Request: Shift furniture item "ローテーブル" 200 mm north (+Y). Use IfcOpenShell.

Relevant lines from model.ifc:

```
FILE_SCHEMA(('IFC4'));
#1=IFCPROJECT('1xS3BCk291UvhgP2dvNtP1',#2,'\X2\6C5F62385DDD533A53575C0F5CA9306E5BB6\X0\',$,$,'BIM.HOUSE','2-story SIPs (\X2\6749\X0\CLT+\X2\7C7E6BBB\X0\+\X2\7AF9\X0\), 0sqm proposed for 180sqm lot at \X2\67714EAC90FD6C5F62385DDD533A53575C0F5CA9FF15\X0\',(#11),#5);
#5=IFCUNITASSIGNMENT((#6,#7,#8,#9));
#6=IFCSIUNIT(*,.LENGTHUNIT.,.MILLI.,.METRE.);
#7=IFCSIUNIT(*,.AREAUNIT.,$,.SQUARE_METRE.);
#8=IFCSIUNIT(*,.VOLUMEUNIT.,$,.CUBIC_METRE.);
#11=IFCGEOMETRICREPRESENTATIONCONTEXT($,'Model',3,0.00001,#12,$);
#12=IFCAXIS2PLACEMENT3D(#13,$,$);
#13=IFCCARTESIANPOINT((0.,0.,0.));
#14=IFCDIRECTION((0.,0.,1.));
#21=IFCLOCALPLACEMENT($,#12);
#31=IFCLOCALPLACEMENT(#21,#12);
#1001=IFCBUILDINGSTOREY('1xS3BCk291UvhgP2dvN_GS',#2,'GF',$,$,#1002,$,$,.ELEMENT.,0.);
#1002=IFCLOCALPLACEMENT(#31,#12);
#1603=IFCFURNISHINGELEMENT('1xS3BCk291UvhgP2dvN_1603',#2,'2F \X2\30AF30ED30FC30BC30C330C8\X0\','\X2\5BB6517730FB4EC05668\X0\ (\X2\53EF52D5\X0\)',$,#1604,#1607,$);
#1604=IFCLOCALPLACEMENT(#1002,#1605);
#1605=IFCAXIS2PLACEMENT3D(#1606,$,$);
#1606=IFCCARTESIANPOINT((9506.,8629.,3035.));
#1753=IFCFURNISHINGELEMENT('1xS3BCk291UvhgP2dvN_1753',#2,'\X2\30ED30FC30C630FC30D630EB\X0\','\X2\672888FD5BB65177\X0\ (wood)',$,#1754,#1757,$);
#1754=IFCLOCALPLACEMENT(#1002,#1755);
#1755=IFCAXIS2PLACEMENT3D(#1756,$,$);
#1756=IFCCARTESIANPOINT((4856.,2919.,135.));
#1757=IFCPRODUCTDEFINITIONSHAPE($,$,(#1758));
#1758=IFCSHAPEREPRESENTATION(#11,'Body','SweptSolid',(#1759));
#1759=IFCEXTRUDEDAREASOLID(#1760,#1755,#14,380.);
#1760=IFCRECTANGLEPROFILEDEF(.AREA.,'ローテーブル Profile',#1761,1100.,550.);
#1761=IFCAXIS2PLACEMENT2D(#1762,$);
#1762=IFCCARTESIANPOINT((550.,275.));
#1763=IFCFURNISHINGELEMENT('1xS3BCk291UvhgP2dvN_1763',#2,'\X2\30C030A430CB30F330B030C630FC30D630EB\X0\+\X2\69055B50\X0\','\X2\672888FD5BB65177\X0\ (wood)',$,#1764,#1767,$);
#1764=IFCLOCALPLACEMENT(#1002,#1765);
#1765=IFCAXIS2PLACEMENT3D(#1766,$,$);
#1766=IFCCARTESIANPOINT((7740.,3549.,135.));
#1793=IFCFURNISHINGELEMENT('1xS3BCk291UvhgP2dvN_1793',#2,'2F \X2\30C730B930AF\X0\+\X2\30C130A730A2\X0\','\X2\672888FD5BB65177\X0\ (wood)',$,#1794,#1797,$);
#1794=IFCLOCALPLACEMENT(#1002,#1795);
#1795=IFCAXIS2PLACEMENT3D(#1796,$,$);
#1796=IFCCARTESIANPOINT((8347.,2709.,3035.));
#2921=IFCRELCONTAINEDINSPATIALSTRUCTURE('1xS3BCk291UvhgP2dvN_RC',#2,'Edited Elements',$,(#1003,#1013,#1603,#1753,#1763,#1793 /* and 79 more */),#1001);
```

```python
import ifcopenshell
import ifcopenshell.api.geometry
import ifcopenshell.util.placement
import ifcopenshell.util.unit

model = ifcopenshell.open("model.ifc")
unit_scale = ifcopenshell.util.unit.calculate_unit_scale(model)

item = model.by_guid("1xS3BCk291UvhgP2dvN_1753")
matrix = ifcopenshell.util.placement.get_local_placement(item.ObjectPlacement)
matrix[1, 3] += 0.2 / unit_scale
ifcopenshell.api.geometry.edit_object_placement(model, product=item, matrix=matrix, is_si=False)

print(ifcopenshell.util.placement.get_local_placement(item.ObjectPlacement).round(3) + 0.0)

model.write("model_updated.ifc")
```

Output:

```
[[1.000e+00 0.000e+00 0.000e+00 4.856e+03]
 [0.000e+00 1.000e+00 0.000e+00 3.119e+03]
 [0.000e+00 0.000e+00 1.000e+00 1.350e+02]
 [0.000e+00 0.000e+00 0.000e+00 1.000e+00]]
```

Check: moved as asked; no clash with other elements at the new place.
